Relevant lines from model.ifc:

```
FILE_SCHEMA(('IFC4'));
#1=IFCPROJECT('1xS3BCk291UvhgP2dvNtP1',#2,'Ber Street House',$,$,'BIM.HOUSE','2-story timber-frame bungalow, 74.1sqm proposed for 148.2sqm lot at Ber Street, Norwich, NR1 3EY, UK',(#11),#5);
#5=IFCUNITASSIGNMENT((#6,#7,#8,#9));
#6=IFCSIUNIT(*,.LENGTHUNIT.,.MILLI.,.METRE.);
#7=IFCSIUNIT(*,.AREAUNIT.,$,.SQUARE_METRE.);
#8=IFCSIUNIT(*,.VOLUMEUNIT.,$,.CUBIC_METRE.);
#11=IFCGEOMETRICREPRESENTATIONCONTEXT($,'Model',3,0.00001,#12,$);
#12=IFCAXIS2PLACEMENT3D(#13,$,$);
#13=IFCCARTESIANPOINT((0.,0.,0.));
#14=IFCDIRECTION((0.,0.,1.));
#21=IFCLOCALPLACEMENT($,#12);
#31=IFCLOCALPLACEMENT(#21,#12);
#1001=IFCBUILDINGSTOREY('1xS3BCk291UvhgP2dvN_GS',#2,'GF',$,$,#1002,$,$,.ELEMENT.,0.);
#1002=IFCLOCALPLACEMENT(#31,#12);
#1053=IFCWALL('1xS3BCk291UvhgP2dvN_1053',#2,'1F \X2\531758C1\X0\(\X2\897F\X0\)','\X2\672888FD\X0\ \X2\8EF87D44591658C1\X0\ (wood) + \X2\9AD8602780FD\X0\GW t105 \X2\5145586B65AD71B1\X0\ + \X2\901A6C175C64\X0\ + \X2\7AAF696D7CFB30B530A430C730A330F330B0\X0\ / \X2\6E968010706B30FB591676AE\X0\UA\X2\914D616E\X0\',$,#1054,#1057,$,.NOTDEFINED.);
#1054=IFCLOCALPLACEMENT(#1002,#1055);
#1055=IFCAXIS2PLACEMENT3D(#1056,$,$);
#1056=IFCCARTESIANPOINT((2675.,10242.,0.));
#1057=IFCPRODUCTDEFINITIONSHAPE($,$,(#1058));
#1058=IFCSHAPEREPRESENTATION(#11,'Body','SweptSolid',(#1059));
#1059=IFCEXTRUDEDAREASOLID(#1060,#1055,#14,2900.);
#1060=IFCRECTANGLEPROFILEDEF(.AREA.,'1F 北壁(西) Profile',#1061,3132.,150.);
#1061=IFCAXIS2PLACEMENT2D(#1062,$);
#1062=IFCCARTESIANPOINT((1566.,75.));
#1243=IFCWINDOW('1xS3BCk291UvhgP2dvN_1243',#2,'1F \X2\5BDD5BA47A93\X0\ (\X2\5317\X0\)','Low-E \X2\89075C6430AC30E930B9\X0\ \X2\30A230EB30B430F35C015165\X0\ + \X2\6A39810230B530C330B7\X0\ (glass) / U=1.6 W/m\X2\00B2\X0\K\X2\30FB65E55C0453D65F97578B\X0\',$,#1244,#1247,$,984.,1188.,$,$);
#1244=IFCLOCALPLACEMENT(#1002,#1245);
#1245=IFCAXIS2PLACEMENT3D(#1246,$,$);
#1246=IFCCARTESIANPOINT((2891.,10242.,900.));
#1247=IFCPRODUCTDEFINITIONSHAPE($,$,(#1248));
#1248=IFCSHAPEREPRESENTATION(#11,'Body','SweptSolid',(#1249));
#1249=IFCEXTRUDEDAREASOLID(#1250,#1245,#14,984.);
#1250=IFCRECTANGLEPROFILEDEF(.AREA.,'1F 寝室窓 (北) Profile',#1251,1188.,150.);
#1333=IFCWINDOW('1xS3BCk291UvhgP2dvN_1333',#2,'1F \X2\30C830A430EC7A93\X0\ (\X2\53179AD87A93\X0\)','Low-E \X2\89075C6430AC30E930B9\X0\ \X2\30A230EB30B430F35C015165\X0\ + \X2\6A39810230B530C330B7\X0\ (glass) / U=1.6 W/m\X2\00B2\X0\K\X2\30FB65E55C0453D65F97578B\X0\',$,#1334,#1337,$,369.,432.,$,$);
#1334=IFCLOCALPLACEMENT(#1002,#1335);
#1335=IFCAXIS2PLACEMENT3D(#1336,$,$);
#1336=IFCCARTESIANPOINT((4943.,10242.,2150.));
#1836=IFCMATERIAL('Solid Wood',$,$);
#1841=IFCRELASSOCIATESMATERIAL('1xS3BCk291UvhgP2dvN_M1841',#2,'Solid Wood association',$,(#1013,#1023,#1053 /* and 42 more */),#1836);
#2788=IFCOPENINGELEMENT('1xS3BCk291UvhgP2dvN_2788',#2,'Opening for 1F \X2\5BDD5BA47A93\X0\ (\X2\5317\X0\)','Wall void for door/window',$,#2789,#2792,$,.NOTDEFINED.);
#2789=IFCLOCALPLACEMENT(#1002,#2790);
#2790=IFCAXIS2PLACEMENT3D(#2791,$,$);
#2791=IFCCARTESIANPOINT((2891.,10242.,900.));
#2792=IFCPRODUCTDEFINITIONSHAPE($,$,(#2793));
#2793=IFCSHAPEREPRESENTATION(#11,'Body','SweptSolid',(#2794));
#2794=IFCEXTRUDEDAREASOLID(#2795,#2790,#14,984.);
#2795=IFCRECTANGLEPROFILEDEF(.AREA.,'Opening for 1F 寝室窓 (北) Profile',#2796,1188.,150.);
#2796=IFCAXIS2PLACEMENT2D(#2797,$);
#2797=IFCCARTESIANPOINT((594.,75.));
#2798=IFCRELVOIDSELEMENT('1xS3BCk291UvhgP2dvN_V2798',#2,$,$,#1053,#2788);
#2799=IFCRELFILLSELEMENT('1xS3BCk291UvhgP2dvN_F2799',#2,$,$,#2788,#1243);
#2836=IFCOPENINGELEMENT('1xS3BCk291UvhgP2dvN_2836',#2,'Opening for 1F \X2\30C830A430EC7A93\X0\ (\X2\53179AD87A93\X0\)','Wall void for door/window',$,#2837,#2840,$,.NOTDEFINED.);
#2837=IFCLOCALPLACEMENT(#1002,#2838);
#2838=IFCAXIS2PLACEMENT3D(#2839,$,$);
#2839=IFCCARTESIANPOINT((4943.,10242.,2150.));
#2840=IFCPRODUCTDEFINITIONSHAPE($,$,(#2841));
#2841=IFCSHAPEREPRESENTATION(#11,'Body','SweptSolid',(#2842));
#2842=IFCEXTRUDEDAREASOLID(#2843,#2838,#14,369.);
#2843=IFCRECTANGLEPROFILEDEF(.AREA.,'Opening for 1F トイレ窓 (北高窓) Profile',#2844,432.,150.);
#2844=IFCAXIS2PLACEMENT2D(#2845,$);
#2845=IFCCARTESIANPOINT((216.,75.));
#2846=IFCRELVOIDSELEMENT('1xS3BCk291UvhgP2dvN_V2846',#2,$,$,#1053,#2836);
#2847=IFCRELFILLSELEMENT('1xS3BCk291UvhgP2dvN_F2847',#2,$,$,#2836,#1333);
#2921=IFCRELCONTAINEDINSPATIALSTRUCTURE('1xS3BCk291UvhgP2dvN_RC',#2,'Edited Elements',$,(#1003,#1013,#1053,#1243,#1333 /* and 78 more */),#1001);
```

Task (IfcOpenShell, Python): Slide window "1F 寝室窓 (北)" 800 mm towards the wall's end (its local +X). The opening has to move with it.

```python
import ifcopenshell
import ifcopenshell.api.geometry
import ifcopenshell.util.placement
import ifcopenshell.util.unit

model = ifcopenshell.open("model.ifc")
unit_scale = ifcopenshell.util.unit.calculate_unit_scale(model)

window = model.by_id(1243)
opening = window.FillsVoids[0].RelatingOpeningElement
wall = opening.VoidsElements[0].RelatingBuildingElement

wall_matrix = ifcopenshell.util.placement.get_local_placement(wall.ObjectPlacement)
shift = wall_matrix[:3, 0] * 0.8 / unit_scale
before = ifcopenshell.util.placement.get_local_placement(window.ObjectPlacement)[:3, 3].copy()

# The window is not placed relative to its opening, so move both.
for product in (opening, window):
    matrix = ifcopenshell.util.placement.get_local_placement(product.ObjectPlacement)
    matrix[:3, 3] += shift
    ifcopenshell.api.geometry.edit_object_placement(model, product=product, matrix=matrix, is_si=False)

after = ifcopenshell.util.placement.get_local_placement(window.ObjectPlacement)[:3, 3]
print("window moved by", (after - before).round(3) + 0.0)

model.write("model-out.ifc")
```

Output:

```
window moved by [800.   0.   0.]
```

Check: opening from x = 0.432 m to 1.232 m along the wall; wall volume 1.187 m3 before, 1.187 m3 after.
